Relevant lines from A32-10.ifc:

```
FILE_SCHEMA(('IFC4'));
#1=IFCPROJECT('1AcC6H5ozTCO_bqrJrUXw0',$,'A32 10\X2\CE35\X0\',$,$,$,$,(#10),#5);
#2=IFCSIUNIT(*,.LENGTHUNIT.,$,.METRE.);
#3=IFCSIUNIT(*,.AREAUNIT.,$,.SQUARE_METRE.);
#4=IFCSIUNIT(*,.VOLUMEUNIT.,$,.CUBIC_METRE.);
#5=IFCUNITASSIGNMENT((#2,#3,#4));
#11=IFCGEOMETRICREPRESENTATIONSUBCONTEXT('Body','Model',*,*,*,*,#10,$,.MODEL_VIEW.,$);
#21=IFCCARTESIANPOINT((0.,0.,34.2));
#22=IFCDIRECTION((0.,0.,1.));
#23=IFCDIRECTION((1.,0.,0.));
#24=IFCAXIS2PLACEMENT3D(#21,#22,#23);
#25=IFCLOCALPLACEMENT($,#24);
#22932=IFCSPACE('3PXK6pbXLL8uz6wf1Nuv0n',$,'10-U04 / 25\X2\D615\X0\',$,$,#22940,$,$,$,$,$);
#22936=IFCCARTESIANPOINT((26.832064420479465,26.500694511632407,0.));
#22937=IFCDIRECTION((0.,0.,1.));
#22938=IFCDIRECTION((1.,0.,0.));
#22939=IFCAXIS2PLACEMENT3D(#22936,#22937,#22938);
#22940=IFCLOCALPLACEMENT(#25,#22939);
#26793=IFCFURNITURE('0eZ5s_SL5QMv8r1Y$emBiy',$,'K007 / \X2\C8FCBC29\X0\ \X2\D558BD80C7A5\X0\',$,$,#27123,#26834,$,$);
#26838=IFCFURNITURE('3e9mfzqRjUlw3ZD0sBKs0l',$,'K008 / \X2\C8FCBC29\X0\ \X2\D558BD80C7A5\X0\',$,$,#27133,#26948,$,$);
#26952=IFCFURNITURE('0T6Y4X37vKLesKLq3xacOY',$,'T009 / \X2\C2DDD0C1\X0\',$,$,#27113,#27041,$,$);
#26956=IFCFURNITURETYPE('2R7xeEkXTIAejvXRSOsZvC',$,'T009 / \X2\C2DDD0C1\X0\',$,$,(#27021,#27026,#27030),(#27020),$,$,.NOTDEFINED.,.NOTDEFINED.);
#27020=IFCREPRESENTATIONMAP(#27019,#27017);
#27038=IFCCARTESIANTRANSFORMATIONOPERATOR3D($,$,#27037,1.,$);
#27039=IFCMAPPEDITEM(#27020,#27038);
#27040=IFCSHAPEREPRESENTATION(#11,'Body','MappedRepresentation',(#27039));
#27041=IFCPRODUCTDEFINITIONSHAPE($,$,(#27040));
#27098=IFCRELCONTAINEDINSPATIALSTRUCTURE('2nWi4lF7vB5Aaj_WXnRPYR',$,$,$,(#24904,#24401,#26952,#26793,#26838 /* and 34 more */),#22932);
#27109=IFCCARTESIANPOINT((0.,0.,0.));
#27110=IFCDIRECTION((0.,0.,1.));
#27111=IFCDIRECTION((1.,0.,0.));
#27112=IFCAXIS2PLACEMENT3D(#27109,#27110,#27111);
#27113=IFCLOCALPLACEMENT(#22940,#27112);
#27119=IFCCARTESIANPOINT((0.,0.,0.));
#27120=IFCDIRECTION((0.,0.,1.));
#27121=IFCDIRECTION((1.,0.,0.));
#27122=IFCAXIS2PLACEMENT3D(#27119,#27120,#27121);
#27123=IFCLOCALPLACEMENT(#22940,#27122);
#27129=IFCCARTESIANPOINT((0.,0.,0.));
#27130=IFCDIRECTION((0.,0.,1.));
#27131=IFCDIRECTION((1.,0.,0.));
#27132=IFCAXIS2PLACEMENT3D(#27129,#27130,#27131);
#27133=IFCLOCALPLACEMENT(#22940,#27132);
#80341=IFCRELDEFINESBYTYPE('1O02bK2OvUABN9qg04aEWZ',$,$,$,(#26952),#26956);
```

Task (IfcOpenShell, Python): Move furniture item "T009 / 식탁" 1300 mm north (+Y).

```python
import ifcopenshell
import ifcopenshell.api.geometry
import ifcopenshell.util.placement
import ifcopenshell.util.unit

model = ifcopenshell.open("A32-10.ifc")
unit_scale = ifcopenshell.util.unit.calculate_unit_scale(model)

item = model.by_guid("0T6Y4X37vKLesKLq3xacOY")
matrix = ifcopenshell.util.placement.get_local_placement(item.ObjectPlacement)
matrix[1, 3] += 1.3 / unit_scale
ifcopenshell.api.geometry.edit_object_placement(model, product=item, matrix=matrix, is_si=False)

print(ifcopenshell.util.placement.get_local_placement(item.ObjectPlacement).round(3) + 0.0)

model.write("A32-10-out.ifc")
```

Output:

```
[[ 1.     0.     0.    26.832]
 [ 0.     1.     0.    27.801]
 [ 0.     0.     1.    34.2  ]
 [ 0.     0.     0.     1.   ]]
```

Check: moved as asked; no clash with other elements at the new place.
